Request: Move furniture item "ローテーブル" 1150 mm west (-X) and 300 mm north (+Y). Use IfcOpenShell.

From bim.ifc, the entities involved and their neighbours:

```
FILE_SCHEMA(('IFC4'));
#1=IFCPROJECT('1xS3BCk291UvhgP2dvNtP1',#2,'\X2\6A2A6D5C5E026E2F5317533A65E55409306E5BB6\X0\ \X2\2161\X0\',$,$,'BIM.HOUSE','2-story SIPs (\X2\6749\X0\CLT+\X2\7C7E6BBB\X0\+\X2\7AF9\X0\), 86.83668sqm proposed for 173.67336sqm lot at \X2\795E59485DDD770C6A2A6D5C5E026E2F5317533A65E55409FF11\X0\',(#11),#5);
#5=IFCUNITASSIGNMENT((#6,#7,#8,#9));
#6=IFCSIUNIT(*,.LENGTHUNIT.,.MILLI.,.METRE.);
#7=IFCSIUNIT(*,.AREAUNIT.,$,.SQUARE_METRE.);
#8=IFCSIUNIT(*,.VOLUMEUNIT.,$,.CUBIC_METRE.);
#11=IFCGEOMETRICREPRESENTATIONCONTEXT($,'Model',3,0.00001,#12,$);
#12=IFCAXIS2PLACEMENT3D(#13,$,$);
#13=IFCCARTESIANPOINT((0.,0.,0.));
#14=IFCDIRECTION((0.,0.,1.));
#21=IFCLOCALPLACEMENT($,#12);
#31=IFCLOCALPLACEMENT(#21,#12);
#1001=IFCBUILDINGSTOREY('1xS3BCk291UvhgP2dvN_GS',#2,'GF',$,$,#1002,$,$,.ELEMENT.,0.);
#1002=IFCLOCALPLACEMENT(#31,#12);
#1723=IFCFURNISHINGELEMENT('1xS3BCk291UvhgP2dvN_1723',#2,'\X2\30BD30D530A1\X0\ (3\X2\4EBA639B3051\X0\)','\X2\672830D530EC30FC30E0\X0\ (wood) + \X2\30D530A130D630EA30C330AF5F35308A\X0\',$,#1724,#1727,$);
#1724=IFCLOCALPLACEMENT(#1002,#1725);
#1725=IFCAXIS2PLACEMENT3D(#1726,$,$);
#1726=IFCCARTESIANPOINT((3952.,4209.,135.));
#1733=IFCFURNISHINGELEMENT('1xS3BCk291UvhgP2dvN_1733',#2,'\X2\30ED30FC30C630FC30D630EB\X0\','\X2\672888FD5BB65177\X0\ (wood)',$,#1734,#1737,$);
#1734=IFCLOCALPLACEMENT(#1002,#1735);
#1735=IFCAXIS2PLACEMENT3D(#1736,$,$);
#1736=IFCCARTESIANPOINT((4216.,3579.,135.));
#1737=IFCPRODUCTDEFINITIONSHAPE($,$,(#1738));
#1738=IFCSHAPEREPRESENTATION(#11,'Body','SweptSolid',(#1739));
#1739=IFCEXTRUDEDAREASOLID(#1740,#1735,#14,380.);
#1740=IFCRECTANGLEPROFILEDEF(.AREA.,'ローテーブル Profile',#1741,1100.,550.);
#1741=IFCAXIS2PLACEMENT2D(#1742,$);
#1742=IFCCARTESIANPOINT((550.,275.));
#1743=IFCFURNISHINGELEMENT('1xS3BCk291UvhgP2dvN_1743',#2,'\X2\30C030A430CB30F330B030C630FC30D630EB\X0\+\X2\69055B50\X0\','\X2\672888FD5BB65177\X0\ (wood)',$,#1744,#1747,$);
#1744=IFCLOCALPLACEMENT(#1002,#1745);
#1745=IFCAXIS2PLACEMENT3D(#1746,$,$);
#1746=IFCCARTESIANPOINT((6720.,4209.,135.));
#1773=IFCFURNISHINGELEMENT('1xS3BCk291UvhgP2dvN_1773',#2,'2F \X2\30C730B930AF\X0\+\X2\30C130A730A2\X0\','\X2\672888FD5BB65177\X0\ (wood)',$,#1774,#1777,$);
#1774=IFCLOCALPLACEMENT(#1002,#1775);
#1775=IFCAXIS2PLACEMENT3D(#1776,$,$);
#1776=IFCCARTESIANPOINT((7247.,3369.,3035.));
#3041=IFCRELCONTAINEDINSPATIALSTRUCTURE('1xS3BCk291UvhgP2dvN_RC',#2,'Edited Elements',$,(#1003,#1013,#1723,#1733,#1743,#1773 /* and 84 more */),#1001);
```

```python
import ifcopenshell
import ifcopenshell.api.geometry
import ifcopenshell.util.placement

model = ifcopenshell.open("bim.ifc")

item = model.by_guid("1xS3BCk291UvhgP2dvN_1733")
matrix = ifcopenshell.util.placement.get_local_placement(item.ObjectPlacement)
matrix[0, 3] -= 1150.0
matrix[1, 3] += 300.0
ifcopenshell.api.geometry.edit_object_placement(model, product=item, matrix=matrix, is_si=False)

print(ifcopenshell.util.placement.get_local_placement(item.ObjectPlacement).round(3) + 0.0)

model.write("bim_edited.ifc")
```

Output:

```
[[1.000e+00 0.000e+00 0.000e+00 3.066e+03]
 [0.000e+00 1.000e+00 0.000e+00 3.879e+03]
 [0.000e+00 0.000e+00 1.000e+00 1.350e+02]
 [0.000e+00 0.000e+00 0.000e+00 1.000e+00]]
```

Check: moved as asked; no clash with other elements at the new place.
